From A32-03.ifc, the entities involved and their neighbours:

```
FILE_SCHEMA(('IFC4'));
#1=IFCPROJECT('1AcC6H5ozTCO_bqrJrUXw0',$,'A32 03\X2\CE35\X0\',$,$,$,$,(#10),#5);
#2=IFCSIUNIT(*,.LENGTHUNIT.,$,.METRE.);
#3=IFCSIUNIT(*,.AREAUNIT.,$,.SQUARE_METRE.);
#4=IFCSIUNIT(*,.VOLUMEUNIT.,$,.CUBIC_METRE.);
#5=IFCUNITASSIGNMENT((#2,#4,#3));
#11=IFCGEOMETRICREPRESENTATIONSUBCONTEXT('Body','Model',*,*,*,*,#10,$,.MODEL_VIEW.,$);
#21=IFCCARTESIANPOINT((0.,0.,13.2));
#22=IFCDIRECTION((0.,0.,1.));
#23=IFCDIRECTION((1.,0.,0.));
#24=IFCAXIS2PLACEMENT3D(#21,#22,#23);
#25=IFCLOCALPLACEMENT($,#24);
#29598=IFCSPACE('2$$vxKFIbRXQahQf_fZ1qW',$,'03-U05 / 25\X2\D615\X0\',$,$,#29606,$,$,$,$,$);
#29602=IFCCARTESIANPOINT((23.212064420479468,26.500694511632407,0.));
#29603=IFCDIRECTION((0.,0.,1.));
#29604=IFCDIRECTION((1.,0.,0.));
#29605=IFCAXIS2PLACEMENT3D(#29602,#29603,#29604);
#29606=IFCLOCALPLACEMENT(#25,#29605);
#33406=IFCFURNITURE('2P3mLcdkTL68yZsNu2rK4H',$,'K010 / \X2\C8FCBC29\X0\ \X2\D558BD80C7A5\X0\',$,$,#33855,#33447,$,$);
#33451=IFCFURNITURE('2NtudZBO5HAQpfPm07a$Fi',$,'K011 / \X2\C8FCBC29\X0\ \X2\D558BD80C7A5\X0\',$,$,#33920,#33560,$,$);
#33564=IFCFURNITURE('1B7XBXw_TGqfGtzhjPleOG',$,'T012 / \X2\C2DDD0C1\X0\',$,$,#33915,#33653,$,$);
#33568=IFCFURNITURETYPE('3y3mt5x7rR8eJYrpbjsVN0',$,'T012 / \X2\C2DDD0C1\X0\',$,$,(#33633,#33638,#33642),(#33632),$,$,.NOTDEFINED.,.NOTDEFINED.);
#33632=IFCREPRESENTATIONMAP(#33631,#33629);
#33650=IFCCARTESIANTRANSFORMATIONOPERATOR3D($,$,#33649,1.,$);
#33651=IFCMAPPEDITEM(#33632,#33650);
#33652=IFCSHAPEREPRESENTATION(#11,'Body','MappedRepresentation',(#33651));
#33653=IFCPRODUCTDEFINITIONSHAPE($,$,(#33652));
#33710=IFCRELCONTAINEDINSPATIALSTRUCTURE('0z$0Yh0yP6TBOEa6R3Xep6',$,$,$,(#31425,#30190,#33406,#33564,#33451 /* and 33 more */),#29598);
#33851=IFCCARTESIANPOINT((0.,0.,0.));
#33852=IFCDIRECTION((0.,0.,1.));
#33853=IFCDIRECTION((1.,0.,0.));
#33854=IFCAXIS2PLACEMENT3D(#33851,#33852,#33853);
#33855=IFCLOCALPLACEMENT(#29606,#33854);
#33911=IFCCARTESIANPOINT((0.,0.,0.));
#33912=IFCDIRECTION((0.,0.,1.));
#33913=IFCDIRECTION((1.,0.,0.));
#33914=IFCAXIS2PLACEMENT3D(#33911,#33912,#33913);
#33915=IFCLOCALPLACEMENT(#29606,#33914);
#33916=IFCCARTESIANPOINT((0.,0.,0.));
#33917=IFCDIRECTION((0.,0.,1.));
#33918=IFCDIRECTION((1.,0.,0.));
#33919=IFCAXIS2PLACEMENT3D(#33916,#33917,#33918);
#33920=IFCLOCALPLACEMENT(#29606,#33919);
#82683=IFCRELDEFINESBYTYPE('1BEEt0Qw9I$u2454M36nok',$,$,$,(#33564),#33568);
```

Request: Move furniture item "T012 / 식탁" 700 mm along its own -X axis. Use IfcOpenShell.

```python
import ifcopenshell
import ifcopenshell.api.geometry
import ifcopenshell.util.placement
import ifcopenshell.util.unit

model = ifcopenshell.open("A32-03.ifc")
unit_scale = ifcopenshell.util.unit.calculate_unit_scale(model)

item = model.by_guid("1B7XBXw_TGqfGtzhjPleOG")
matrix = ifcopenshell.util.placement.get_local_placement(item.ObjectPlacement)
matrix[:3, 3] -= matrix[:3, 0] * 0.7 / unit_scale
ifcopenshell.api.geometry.edit_object_placement(model, product=item, matrix=matrix, is_si=False)

print(ifcopenshell.util.placement.get_local_placement(item.ObjectPlacement).round(3) + 0.0)

model.write("A32-03_v2.ifc")
```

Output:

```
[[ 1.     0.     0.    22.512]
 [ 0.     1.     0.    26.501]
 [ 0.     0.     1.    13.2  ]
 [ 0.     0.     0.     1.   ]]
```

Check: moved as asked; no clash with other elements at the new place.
